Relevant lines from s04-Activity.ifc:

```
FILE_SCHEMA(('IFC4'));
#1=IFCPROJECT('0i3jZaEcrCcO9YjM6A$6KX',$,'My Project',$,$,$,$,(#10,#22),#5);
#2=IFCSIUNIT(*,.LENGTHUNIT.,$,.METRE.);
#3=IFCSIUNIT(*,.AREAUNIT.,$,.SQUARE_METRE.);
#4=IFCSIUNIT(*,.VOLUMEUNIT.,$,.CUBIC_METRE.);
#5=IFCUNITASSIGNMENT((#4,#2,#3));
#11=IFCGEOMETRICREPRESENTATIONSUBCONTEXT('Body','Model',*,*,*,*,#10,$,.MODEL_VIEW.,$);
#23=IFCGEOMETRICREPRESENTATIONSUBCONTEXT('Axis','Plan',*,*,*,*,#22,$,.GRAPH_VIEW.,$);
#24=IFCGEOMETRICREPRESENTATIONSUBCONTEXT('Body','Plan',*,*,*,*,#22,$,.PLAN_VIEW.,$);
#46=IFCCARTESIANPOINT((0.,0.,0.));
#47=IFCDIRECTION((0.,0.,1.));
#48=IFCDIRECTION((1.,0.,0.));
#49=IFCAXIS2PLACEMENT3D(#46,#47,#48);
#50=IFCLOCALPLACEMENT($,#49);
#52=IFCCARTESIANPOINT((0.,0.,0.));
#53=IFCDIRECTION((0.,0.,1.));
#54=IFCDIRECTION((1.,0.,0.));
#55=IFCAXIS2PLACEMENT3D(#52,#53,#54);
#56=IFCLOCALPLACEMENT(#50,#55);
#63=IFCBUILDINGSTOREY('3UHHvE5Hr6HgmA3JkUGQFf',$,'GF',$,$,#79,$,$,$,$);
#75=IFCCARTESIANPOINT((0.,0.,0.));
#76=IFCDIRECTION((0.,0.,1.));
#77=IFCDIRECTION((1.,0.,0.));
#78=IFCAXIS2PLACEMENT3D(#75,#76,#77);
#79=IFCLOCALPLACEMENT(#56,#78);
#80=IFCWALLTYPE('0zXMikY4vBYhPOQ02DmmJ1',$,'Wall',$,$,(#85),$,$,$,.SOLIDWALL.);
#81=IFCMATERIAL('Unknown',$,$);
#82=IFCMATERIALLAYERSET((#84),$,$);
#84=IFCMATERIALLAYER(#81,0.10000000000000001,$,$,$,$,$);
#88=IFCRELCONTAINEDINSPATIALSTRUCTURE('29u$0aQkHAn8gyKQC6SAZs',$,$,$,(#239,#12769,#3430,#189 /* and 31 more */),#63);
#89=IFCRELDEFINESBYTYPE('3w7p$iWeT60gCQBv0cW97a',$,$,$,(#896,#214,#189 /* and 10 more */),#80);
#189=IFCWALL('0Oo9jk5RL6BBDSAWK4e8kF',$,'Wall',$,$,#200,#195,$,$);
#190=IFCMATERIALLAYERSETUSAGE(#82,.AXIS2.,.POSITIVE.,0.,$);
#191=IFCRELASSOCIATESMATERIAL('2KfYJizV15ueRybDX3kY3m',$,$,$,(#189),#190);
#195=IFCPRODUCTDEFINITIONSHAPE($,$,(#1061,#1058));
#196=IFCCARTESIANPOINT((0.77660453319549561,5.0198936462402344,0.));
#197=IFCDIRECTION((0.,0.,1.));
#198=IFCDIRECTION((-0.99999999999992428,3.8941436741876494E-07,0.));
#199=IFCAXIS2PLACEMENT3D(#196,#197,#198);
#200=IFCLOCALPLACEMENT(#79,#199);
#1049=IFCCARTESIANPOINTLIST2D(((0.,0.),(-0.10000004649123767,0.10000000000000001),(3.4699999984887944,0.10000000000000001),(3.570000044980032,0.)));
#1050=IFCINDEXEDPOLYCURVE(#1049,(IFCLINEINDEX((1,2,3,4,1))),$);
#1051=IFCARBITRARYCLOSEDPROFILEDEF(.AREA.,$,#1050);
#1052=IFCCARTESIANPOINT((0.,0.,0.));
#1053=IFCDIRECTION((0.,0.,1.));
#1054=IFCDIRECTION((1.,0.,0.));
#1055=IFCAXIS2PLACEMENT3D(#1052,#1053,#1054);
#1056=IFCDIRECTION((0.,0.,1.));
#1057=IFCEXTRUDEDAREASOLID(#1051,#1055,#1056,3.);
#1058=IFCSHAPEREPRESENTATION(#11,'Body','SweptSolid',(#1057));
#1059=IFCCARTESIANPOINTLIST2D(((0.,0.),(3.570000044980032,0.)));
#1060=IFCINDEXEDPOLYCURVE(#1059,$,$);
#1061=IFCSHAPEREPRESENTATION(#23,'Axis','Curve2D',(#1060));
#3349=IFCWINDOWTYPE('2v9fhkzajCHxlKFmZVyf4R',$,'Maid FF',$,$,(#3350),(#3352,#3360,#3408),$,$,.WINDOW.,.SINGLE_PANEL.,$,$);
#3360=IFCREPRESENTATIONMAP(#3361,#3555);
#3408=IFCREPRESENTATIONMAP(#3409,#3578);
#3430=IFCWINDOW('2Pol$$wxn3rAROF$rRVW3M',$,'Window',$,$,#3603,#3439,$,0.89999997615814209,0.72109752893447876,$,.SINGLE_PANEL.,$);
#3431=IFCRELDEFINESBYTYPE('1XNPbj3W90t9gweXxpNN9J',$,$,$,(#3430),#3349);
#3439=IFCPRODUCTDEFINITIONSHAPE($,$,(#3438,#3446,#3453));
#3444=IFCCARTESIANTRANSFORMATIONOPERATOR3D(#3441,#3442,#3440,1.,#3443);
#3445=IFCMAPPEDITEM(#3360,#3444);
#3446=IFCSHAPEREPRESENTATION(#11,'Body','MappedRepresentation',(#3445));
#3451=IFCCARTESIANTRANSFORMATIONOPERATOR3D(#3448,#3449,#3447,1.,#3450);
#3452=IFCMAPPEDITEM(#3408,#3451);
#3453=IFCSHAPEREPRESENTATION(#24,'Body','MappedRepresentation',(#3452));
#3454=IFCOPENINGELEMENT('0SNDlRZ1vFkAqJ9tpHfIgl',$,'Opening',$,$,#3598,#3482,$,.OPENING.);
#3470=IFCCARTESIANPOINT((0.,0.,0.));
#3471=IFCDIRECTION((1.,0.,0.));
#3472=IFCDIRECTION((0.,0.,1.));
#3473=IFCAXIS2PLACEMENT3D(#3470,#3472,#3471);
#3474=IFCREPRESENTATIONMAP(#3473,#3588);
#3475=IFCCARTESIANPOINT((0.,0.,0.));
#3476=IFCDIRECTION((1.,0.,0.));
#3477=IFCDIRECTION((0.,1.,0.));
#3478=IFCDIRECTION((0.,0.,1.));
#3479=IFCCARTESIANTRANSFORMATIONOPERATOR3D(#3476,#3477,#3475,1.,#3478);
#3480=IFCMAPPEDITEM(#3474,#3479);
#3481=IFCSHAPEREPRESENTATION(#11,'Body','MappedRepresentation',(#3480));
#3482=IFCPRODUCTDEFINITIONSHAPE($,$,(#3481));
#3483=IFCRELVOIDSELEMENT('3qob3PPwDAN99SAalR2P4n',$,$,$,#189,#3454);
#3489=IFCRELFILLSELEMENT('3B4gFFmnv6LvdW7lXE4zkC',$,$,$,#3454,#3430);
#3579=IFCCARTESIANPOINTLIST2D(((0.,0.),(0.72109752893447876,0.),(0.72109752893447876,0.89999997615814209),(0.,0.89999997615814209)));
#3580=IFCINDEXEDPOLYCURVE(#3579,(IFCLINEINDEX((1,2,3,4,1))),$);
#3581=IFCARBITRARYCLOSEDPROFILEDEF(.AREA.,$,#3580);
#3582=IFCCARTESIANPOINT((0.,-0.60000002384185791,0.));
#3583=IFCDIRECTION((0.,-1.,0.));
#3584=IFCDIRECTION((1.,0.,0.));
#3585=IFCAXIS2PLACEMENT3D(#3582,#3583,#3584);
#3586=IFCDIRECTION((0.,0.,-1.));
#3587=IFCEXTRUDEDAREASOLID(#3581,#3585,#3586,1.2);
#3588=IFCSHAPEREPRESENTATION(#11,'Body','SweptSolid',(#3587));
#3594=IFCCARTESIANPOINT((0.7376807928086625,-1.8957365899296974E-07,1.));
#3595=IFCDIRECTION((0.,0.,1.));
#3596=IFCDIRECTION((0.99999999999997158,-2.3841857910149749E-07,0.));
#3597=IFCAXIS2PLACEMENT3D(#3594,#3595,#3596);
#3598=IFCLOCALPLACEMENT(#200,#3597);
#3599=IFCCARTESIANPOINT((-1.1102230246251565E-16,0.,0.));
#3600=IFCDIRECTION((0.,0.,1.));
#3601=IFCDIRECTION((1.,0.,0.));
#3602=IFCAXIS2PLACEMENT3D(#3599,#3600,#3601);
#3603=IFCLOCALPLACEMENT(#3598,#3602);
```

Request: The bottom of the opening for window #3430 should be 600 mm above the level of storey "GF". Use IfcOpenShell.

```python
import numpy as np
import ifcopenshell
import ifcopenshell.api.geometry
import ifcopenshell.geom
import ifcopenshell.util.element
import ifcopenshell.util.placement
import ifcopenshell.util.shape
import ifcopenshell.util.unit

model = ifcopenshell.open("s04-Activity.ifc")
unit_scale = ifcopenshell.util.unit.calculate_unit_scale(model)

window = model.by_id(3430)
opening = window.FillsVoids[0].RelatingOpeningElement
storey = ifcopenshell.util.element.get_container(window, ifc_class="IfcBuildingStorey")
level = ifcopenshell.util.placement.get_local_placement(storey.ObjectPlacement)[2, 3]

# The opening's origin need not be at the sill, so measure its lowest point.
shape = ifcopenshell.geom.create_shape(ifcopenshell.geom.settings(), opening)
bottom = ifcopenshell.util.shape.get_shape_bottom_elevation(shape, shape.geometry) / unit_scale
dz = level + 0.6 - bottom

shift = np.array([0.0, 0.0, dz])
# The window is placed relative to its opening, so it follows when the opening moves.
matrix = ifcopenshell.util.placement.get_local_placement(opening.ObjectPlacement)
matrix[:3, 3] += shift
ifcopenshell.api.geometry.edit_object_placement(
    model, product=opening, matrix=matrix, is_si=False, should_transform_children=True
)

print(f"moved by {dz * unit_scale:+.3f} m")

model.write("s04-Activity_edited.ifc")
```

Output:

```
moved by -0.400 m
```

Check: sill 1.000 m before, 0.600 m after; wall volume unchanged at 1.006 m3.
